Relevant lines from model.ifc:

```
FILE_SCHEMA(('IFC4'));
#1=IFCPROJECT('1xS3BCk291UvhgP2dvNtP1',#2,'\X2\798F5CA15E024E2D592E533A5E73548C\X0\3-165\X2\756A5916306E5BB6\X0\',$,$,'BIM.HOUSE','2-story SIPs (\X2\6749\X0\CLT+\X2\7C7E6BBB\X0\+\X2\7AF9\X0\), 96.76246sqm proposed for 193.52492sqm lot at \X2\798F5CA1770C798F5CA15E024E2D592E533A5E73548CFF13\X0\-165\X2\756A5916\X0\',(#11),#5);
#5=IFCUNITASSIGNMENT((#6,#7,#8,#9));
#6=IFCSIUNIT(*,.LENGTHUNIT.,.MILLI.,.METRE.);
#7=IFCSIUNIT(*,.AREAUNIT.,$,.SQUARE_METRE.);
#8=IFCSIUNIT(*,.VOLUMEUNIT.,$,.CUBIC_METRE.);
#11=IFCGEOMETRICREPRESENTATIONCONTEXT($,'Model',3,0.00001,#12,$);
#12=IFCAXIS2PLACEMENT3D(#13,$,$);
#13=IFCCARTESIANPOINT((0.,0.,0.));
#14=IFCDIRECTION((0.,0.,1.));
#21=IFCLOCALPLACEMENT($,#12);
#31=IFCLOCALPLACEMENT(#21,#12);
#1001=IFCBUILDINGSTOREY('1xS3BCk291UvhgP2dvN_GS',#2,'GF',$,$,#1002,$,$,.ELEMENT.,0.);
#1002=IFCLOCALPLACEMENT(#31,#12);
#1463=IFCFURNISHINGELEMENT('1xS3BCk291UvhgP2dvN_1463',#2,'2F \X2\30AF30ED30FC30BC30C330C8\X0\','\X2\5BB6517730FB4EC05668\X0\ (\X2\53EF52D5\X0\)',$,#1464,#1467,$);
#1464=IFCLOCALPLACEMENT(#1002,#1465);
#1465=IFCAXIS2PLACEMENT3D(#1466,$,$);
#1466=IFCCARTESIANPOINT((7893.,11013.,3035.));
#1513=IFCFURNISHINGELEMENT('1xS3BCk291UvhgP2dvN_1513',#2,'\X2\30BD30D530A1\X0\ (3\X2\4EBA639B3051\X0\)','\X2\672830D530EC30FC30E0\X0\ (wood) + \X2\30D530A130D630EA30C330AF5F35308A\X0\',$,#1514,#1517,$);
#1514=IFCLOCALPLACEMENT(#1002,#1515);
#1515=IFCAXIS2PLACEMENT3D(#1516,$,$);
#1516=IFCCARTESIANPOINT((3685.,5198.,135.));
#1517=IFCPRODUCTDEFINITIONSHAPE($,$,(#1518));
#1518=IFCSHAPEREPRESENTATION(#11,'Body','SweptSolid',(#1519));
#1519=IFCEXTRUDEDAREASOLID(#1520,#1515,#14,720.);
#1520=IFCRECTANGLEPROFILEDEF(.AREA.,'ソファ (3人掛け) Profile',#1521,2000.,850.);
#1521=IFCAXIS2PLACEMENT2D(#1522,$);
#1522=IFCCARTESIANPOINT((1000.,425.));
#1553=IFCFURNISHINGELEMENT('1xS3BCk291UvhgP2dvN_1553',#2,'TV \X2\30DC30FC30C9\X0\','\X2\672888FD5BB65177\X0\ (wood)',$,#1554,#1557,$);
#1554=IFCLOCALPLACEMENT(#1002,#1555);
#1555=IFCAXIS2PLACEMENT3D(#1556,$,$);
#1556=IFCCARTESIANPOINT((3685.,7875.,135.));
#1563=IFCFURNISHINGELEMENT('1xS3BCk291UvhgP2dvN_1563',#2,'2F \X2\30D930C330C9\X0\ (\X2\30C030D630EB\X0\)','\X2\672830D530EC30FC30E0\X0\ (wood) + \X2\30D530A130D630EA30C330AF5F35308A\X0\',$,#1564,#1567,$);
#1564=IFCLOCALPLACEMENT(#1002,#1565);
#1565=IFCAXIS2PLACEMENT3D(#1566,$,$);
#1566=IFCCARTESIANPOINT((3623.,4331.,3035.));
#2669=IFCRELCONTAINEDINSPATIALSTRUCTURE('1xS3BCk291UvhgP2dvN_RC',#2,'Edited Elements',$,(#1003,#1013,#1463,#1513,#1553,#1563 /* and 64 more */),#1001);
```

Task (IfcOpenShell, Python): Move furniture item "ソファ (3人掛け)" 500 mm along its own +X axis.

```python
import ifcopenshell
import ifcopenshell.api.geometry
import ifcopenshell.util.placement
import ifcopenshell.util.unit

model = ifcopenshell.open("model.ifc")
unit_scale = ifcopenshell.util.unit.calculate_unit_scale(model)

item = model.by_guid("1xS3BCk291UvhgP2dvN_1513")
matrix = ifcopenshell.util.placement.get_local_placement(item.ObjectPlacement)
matrix[:3, 3] += matrix[:3, 0] * 0.5 / unit_scale
ifcopenshell.api.geometry.edit_object_placement(model, product=item, matrix=matrix, is_si=False)

print(ifcopenshell.util.placement.get_local_placement(item.ObjectPlacement).round(3) + 0.0)

model.write("model_v2.ifc")
```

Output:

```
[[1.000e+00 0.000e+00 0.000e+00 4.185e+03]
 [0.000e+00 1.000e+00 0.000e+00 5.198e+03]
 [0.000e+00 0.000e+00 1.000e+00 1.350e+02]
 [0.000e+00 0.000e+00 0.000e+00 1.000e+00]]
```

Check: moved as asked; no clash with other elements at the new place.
